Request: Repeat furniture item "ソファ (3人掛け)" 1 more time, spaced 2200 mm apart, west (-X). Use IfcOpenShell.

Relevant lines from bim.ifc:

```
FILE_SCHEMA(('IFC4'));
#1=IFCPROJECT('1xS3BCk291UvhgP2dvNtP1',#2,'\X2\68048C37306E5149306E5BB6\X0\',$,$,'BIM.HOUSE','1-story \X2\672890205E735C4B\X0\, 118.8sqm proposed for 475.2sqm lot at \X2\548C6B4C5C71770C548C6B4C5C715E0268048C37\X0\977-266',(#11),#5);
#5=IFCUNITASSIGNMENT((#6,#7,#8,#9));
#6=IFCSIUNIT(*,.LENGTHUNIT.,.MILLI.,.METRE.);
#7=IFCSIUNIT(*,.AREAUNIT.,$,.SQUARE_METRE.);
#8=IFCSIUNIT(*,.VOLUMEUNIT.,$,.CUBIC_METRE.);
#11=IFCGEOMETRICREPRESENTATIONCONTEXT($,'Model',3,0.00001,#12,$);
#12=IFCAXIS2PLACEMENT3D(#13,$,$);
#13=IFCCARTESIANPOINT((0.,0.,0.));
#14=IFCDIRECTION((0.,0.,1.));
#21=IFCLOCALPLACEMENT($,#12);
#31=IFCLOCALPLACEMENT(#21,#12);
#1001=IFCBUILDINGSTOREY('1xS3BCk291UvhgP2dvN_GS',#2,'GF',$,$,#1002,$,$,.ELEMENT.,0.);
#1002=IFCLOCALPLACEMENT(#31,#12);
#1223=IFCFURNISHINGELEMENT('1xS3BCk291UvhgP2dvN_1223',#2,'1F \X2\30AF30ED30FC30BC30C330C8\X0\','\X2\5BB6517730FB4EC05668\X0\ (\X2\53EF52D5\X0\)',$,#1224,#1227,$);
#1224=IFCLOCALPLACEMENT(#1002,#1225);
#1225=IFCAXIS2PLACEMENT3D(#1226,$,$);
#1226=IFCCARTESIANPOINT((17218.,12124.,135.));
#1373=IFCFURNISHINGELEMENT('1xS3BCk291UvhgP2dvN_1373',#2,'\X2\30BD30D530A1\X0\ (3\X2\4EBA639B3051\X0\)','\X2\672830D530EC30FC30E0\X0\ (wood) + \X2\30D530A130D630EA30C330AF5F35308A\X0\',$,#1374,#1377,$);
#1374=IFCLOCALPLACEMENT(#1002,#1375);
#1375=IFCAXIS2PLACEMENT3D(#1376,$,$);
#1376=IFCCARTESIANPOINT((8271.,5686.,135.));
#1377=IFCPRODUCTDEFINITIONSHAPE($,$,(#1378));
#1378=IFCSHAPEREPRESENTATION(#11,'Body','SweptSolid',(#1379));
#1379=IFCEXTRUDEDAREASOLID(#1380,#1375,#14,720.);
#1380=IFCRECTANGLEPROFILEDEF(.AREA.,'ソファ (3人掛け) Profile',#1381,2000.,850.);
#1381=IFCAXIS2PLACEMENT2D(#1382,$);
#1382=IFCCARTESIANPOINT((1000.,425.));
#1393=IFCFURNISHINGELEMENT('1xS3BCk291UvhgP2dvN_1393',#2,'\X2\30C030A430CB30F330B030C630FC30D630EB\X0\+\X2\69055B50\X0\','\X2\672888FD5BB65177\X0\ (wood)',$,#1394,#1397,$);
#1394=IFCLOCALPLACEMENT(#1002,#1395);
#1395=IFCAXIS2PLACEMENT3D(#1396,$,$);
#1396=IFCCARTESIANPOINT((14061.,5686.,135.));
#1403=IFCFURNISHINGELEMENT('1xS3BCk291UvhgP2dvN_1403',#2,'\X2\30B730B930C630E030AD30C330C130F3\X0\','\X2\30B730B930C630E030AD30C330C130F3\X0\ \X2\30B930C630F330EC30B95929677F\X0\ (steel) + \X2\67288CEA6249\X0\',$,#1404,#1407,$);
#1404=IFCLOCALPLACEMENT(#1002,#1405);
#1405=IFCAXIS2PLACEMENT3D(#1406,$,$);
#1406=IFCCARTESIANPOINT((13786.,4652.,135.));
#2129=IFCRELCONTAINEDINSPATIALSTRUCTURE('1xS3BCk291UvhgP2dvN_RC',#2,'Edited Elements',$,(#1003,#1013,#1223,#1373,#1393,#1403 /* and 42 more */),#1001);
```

```python
import numpy as np
import ifcopenshell
import ifcopenshell.api.geometry
import ifcopenshell.api.root
import ifcopenshell.util.element
import ifcopenshell.util.placement
import ifcopenshell.util.unit

model = ifcopenshell.open("bim.ifc")
unit_scale = ifcopenshell.util.unit.calculate_unit_scale(model)


def reuse_history(source, copy):
    """copy_class also copies each property set's owner history, people and application; keep the originals."""
    for rel in copy.IsDefinedBy:
        if rel.is_a("IfcRelDefinesByProperties") and (history := rel.RelatingPropertyDefinition.OwnerHistory):
            rel.RelatingPropertyDefinition.OwnerHistory = source.OwnerHistory
            ifcopenshell.util.element.remove_deep2(model, history)


source = model.by_guid("1xS3BCk291UvhgP2dvN_1373")
base = ifcopenshell.util.placement.get_local_placement(source.ObjectPlacement)
step = np.array([-1.0, 0.0, 0.0]) * 2.2 / unit_scale

for i in range(1, 2):
    copy = ifcopenshell.api.root.copy_class(model, product=source)
    copy.Representation = ifcopenshell.util.element.copy_deep(
        model, source.Representation, exclude=["IfcGeometricRepresentationContext", "IfcRepresentationMap"]
    )
    reuse_history(source, copy)
    matrix = base.copy()
    matrix[:3, 3] += i * step
    print("added at", matrix[:3, 3].round(3) + 0.0)
    ifcopenshell.api.geometry.edit_object_placement(model, product=copy, matrix=matrix, is_si=False)

model.write("bim_updated.ifc")
```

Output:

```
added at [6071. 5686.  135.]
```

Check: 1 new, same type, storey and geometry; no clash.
